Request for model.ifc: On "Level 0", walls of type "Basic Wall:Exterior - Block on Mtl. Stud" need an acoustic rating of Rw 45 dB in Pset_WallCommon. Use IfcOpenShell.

First a look at what the model holds.

```python
import ifcopenshell
import ifcopenshell.util.element

model = ifcopenshell.open("model.ifc")
print(model.schema)
storey = next(s for s in model.by_type("IfcBuildingStorey") if s.Name == "Level 0")
walls = [e for e in ifcopenshell.util.element.get_decomposition(storey) if e.is_a("IfcWall")]
seen = {}
for e in walls:
    element_type = ifcopenshell.util.element.get_type(e)
    key = (element_type.Name if element_type != e and element_type else None, ifcopenshell.util.element.get_pset(e, "Pset_WallCommon", "AcousticRating"))
    seen[key] = seen.get(key, 0) + 1
for (name, value), count in sorted(seen.items(), key=str):
    print(count, "x", name, "|", value)
```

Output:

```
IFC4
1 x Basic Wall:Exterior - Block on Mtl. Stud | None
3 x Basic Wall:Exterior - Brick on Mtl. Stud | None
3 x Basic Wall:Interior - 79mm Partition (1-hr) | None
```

```python
import ifcopenshell
import ifcopenshell.api.pset
import ifcopenshell.util.element

model = ifcopenshell.open("model.ifc")

storey = next(s for s in model.by_type("IfcBuildingStorey") if s.Name == "Level 0")
walls = [e for e in ifcopenshell.util.element.get_decomposition(storey) if e.is_a("IfcWall")]

count = 0
for e in walls:
    element_type = ifcopenshell.util.element.get_type(e)
    if element_type in (None, e) or element_type.Name != "Basic Wall:Exterior - Block on Mtl. Stud":
        continue
    # add_pset returns the element's existing set when there is one.
    pset = ifcopenshell.api.pset.add_pset(model, product=e, name="Pset_WallCommon")
    ifcopenshell.api.pset.edit_pset(model, pset=pset, properties={"AcousticRating": "Rw 45 dB"})
    count += 1

print(count, "walls updated")

model.write("model_rev.ifc")
```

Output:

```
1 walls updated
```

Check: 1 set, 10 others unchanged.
